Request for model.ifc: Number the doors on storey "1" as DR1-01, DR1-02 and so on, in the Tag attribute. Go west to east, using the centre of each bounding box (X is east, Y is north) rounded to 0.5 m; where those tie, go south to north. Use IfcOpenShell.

First a look at what the model holds.

```python
import ifcopenshell
import ifcopenshell.util.element
import ifcopenshell.util.placement

model = ifcopenshell.open("model.ifc")
print(model.schema)
storey = next(s for s in model.by_type("IfcBuildingStorey") if s.Name == "1")
doors = [e for e in ifcopenshell.util.element.get_decomposition(storey) if e.is_a("IfcDoor")]
for e in sorted(doors, key=lambda e: e.id()):
    origin = ifcopenshell.util.placement.get_local_placement(e.ObjectPlacement)[:3, 3]
    print(e.id(), e.Tag, e.Name, origin.round(2) + 0.0, sep=" | ")
```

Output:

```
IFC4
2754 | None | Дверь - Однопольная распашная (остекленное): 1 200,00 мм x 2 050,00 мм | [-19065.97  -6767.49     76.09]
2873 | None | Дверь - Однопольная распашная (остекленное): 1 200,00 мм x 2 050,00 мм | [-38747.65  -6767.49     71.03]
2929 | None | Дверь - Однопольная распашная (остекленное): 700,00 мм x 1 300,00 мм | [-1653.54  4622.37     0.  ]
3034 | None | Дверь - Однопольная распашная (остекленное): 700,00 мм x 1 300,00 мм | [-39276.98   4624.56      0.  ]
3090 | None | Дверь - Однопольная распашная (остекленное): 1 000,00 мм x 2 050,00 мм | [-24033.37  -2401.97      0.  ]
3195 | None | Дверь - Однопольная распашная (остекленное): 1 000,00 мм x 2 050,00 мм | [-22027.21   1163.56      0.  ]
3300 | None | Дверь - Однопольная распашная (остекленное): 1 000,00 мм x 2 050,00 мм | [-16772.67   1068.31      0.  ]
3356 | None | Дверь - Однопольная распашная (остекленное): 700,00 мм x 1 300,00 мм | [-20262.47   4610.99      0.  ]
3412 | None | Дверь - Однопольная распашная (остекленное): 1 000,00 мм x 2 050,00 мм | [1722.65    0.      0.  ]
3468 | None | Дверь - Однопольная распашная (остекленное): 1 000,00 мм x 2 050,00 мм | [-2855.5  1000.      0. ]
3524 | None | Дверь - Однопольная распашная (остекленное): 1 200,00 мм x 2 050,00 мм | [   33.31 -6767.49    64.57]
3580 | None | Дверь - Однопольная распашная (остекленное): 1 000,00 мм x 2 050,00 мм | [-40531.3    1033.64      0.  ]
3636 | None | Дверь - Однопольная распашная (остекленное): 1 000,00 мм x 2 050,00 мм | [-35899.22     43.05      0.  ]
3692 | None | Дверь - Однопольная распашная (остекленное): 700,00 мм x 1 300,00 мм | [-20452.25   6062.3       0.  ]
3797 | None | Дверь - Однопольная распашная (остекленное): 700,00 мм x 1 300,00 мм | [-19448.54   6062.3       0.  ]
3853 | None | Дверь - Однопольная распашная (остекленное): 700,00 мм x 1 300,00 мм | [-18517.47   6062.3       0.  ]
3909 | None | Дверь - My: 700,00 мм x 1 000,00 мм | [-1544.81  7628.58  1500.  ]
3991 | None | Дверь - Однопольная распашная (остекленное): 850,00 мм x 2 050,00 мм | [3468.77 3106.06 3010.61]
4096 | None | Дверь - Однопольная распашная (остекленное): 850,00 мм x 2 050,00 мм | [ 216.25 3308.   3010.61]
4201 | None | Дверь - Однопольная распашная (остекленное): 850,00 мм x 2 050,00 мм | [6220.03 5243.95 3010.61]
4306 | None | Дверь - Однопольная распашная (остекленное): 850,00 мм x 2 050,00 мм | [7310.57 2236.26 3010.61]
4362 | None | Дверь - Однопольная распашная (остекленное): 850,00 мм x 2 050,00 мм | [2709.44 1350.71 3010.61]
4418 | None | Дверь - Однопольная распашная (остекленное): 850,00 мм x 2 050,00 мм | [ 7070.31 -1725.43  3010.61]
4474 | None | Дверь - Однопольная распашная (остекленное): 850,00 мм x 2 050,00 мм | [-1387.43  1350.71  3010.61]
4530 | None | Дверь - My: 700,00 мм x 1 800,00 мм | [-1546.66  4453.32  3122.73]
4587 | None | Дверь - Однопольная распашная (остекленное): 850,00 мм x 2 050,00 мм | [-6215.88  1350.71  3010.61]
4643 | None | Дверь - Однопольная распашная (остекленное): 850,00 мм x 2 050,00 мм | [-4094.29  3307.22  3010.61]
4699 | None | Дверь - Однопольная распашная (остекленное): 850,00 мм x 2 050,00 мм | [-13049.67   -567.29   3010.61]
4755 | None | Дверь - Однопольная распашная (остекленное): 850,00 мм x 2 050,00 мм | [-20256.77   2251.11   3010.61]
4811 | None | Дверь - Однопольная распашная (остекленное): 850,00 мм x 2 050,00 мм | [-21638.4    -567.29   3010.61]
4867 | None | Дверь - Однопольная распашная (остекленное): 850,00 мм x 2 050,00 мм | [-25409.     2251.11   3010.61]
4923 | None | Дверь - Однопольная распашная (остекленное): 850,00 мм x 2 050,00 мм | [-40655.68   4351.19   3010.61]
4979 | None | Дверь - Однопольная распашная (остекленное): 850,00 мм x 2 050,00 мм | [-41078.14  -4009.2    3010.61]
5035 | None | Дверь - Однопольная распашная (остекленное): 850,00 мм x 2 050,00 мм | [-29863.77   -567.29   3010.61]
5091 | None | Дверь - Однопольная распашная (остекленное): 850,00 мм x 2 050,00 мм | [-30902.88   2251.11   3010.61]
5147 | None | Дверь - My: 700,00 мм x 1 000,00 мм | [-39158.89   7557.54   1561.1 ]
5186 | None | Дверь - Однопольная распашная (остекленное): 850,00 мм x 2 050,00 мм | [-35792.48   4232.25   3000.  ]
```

```python
import ifcopenshell
import ifcopenshell.geom
import ifcopenshell.util.element
import ifcopenshell.util.shape

model = ifcopenshell.open("model.ifc")
settings = ifcopenshell.geom.settings()
settings.set("use-world-coords", True)


def centre(element):
    shape = ifcopenshell.geom.create_shape(settings, element)
    return ifcopenshell.util.shape.get_bbox_centroid(shape.geometry)


storey = next(s for s in model.by_type("IfcBuildingStorey") if s.Name == "1")
doors = [e for e in ifcopenshell.util.element.get_decomposition(storey) if e.is_a("IfcDoor")]

# Insertion points can sit at a corner or the storey origin, so sort by the geometry (in metres).
centres = {e: centre(e) for e in doors}
doors.sort(key=lambda e: (round(centres[e][0] / 0.5), centres[e][1]))

for i, e in enumerate(doors, start=1):
    number = f"DR1-{i:02d}"
    e.Tag = number
    print(e.id(), number)

model.write("model_rev.ifc")
```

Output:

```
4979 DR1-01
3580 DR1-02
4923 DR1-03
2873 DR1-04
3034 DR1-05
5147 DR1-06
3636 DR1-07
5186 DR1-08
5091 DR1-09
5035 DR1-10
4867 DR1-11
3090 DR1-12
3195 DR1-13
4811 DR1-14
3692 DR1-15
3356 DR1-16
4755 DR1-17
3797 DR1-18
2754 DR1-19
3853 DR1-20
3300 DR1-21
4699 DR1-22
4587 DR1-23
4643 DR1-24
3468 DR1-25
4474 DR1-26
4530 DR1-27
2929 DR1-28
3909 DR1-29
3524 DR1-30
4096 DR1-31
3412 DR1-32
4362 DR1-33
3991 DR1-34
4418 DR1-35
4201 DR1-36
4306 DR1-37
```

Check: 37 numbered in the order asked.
